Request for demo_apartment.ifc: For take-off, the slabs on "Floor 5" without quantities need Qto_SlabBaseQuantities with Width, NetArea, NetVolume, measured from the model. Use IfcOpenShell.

First a look at what the model holds.

```python
import ifcopenshell
import ifcopenshell.util.element
import ifcopenshell.util.unit

model = ifcopenshell.open("demo_apartment.ifc")
print(model.schema)
for unit_type in ("LENGTHUNIT", "AREAUNIT", "VOLUMEUNIT"):
    print(unit_type, ifcopenshell.util.unit.calculate_unit_scale(model, unit_type))
storey = next(s for s in model.by_type("IfcBuildingStorey") if s.Name == "Floor 5")
slabs = [e for e in ifcopenshell.util.element.get_decomposition(storey) if e.is_a("IfcSlab")]
for e in sorted(slabs, key=lambda e: e.id()):
    print(e.id(), e.is_a(), e.Name, list(ifcopenshell.util.element.get_psets(e, qtos_only=True)), sep=" | ")
```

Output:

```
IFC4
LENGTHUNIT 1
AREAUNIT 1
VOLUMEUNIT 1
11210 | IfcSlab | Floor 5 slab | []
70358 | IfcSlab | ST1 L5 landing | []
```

```python
import ifcopenshell
import ifcopenshell.api.pset
import ifcopenshell.geom
import ifcopenshell.util.element
import ifcopenshell.util.shape
import ifcopenshell.util.unit

model = ifcopenshell.open("demo_apartment.ifc")
unit_scale = ifcopenshell.util.unit.calculate_unit_scale(model)
area_scale = ifcopenshell.util.unit.calculate_unit_scale(model, "AREAUNIT")
volume_scale = ifcopenshell.util.unit.calculate_unit_scale(model, "VOLUMEUNIT")
settings = ifcopenshell.geom.settings()

storey = next(s for s in model.by_type("IfcBuildingStorey") if s.Name == "Floor 5")
slabs = [e for e in ifcopenshell.util.element.get_decomposition(storey) if e.is_a("IfcSlab")]

for e in sorted(slabs, key=lambda e: e.id()):
    if ifcopenshell.util.element.get_psets(e, qtos_only=True, should_inherit=False):
        continue
    # Geometry comes back in metres, in the element's own axes.
    shape = ifcopenshell.geom.create_shape(settings, e)
    values = {
        "Width": ifcopenshell.util.shape.get_z(shape.geometry) / unit_scale,
        "NetArea": ifcopenshell.util.shape.get_footprint_area(shape.geometry) / area_scale,
        "NetVolume": ifcopenshell.util.shape.get_volume(shape.geometry) / volume_scale,
    }
    qto = ifcopenshell.api.pset.add_qto(model, product=e, name="Qto_SlabBaseQuantities")
    ifcopenshell.api.pset.edit_qto(model, qto=qto, properties=values)
    print(e.id(), {k: round(v, 3) for k, v in values.items()})

model.write("demo_apartment_v2.ifc")
```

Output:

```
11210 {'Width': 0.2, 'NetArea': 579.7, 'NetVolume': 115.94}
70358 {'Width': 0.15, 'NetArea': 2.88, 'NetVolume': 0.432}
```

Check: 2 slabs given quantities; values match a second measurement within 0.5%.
